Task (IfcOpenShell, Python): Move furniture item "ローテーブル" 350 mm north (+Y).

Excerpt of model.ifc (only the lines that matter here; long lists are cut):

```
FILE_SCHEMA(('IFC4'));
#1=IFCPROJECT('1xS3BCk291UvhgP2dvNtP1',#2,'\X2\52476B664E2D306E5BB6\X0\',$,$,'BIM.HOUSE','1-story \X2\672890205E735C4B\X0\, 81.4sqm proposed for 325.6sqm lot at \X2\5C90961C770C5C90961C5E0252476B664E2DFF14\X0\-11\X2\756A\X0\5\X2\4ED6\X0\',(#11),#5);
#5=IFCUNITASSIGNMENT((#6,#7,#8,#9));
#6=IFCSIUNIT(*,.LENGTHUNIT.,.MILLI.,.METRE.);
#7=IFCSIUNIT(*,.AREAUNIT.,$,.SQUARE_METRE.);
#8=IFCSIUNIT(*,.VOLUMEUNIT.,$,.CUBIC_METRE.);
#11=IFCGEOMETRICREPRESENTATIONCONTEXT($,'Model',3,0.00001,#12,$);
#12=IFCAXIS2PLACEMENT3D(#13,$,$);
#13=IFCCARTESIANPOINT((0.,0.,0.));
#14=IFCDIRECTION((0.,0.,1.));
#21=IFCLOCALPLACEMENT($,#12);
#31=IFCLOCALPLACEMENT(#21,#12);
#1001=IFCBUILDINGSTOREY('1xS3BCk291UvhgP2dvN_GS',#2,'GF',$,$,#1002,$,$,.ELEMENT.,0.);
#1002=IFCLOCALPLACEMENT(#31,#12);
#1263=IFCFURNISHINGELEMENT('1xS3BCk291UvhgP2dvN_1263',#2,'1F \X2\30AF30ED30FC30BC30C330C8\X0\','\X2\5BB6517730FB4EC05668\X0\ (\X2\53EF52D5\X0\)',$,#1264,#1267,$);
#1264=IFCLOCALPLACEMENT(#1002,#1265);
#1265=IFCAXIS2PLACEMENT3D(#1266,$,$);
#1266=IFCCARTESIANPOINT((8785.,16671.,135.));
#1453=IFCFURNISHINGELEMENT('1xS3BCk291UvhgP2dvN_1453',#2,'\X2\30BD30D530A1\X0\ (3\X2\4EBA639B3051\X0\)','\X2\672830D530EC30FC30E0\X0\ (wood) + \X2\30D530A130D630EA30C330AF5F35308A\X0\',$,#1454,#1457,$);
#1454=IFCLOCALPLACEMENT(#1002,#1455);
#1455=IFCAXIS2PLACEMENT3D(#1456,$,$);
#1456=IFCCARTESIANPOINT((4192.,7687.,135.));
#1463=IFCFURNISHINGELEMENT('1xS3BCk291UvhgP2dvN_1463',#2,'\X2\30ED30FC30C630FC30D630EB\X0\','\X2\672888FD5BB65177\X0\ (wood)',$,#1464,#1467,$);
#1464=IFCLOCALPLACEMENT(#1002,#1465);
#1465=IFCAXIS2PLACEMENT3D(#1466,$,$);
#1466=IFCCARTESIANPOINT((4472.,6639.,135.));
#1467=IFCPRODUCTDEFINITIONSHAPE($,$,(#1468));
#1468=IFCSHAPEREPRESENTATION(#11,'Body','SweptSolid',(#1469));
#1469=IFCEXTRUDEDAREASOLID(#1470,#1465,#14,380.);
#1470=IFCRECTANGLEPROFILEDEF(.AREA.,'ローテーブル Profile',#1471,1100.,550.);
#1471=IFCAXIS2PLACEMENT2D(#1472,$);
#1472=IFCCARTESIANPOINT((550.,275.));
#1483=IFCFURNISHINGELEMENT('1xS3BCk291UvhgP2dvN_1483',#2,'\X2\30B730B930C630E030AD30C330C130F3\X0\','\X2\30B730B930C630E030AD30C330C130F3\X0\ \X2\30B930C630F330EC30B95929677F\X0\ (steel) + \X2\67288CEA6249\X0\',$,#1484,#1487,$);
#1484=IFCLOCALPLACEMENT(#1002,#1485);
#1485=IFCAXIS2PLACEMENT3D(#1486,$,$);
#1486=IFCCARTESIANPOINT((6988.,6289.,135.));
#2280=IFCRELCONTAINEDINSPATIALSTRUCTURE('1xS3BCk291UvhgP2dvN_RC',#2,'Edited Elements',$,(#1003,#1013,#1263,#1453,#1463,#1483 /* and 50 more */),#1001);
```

```python
import ifcopenshell
import ifcopenshell.api.geometry
import ifcopenshell.util.placement

model = ifcopenshell.open("model.ifc")

item = model.by_id(1463)
matrix = ifcopenshell.util.placement.get_local_placement(item.ObjectPlacement)
matrix[1, 3] += 350.0
ifcopenshell.api.geometry.edit_object_placement(model, product=item, matrix=matrix, is_si=False)

print(ifcopenshell.util.placement.get_local_placement(item.ObjectPlacement).round(3) + 0.0)

model.write("model_edited.ifc")
```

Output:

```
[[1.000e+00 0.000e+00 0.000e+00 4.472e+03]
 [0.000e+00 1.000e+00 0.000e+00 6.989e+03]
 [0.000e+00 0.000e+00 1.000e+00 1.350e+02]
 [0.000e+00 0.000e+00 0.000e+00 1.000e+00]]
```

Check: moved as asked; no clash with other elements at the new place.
